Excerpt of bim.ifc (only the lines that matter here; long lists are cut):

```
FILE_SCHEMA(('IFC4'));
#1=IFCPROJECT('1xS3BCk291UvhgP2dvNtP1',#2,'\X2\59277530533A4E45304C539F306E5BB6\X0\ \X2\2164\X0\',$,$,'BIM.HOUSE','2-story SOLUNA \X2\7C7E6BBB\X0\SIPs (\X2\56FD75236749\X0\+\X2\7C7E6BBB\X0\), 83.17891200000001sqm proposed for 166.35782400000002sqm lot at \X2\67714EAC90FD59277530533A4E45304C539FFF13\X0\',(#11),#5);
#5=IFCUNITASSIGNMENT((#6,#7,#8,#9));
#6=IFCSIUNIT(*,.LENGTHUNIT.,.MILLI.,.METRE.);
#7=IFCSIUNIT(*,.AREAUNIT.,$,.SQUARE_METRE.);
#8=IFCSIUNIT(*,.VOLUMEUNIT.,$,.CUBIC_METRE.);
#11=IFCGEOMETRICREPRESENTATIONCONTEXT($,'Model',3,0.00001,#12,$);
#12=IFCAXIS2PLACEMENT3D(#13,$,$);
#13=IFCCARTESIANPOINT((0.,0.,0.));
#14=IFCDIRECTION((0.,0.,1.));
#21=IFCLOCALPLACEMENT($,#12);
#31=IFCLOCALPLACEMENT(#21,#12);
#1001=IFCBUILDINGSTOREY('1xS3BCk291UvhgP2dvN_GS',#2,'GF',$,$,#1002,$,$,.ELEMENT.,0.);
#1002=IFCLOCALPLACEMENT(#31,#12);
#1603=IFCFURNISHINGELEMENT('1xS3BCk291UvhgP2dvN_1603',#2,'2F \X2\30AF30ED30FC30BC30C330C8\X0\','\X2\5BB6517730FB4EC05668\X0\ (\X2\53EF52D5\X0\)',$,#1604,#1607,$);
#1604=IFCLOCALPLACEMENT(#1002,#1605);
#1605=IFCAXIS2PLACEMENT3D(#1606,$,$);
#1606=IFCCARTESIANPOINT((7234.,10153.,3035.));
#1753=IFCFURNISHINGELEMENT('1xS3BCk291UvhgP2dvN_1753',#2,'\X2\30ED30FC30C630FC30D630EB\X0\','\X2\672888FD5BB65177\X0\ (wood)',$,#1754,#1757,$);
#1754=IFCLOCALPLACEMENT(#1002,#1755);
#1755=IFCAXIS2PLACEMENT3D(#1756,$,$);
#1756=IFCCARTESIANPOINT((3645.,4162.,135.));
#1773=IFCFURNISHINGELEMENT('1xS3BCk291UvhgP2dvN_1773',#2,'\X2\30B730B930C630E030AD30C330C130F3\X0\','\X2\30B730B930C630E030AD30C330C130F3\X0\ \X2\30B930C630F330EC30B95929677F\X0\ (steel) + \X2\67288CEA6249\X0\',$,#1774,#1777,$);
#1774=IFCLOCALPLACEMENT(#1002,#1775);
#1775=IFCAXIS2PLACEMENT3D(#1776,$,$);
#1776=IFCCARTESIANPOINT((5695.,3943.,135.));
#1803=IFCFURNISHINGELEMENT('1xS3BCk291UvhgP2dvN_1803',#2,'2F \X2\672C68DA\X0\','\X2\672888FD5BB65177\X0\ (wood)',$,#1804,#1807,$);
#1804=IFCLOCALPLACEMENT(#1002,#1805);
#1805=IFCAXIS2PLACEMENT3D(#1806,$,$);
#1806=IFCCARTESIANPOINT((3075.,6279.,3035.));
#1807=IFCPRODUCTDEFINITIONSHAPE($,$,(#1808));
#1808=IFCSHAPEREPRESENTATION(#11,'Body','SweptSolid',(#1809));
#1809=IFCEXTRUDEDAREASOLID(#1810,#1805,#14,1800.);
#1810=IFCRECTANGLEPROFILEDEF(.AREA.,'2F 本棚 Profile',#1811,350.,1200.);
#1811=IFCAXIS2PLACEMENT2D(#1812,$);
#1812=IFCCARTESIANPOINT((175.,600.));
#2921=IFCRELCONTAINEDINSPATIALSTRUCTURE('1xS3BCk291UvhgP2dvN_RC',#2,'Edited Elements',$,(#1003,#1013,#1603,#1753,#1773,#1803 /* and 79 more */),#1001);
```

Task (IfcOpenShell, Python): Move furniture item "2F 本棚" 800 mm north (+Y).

```python
import ifcopenshell
import ifcopenshell.api.geometry
import ifcopenshell.util.placement

model = ifcopenshell.open("bim.ifc")

item = model.by_guid("1xS3BCk291UvhgP2dvN_1803")
matrix = ifcopenshell.util.placement.get_local_placement(item.ObjectPlacement)
matrix[1, 3] += 800.0
ifcopenshell.api.geometry.edit_object_placement(model, product=item, matrix=matrix, is_si=False)

print(ifcopenshell.util.placement.get_local_placement(item.ObjectPlacement).round(3) + 0.0)

model.write("bim_v2.ifc")
```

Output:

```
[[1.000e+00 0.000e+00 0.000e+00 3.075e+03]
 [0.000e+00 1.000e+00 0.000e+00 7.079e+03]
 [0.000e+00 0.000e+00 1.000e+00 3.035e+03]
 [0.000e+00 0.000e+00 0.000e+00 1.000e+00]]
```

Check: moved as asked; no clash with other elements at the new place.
